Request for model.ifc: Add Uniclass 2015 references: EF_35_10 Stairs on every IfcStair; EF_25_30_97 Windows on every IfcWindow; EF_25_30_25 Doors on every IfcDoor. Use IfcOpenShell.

First a look at what the model holds.

```python
import ifcopenshell

model = ifcopenshell.open("model.ifc")
print(model.schema)
print("classifications:", [c.Name for c in model.by_type("IfcClassification")])
for ifc_class in ("IfcDoor", "IfcRoof", "IfcStair", "IfcWall", "IfcWindow"):
    print(ifc_class, len(model.by_type(ifc_class)))
```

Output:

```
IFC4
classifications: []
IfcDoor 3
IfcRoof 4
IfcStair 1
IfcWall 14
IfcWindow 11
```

```python
import ifcopenshell
import ifcopenshell.api.classification

model = ifcopenshell.open("model.ifc")

system = ifcopenshell.api.classification.add_classification(model, classification="Uniclass 2015")

codes = {
    "IfcStair": ("EF_35_10", "Stairs"),
    "IfcWindow": ("EF_25_30_97", "Windows"),
    "IfcDoor": ("EF_25_30_25", "Doors"),
}
for ifc_class, (code, name) in codes.items():
    products = model.by_type(ifc_class)
    ifcopenshell.api.classification.add_reference(
        model, products=products, classification=system, identification=code, name=name
    )
    print(code, len(products))

model.write("model_edited.ifc")
```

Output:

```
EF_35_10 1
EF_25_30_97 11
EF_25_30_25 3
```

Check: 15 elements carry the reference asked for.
